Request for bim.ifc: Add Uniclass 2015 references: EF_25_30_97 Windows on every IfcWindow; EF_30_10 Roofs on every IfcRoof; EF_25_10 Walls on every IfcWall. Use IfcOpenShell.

First a look at what the model holds.

```python
import ifcopenshell

model = ifcopenshell.open("bim.ifc")
print(model.schema)
print("classifications:", [c.Name for c in model.by_type("IfcClassification")])
for ifc_class in ("IfcDoor", "IfcRoof", "IfcStair", "IfcWall", "IfcWindow"):
    print(ifc_class, len(model.by_type(ifc_class)))
```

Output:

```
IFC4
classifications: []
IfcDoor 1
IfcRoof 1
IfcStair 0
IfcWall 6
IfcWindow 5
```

```python
import ifcopenshell
import ifcopenshell.api.classification

model = ifcopenshell.open("bim.ifc")

system = ifcopenshell.api.classification.add_classification(model, classification="Uniclass 2015")

codes = {
    "IfcWindow": ("EF_25_30_97", "Windows"),
    "IfcRoof": ("EF_30_10", "Roofs"),
    "IfcWall": ("EF_25_10", "Walls"),
}
for ifc_class, (code, name) in codes.items():
    products = model.by_type(ifc_class)
    ifcopenshell.api.classification.add_reference(
        model, products=products, classification=system, identification=code, name=name
    )
    print(code, len(products))

model.write("bim-out.ifc")
```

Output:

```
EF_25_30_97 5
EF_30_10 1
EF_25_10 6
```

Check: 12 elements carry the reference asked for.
